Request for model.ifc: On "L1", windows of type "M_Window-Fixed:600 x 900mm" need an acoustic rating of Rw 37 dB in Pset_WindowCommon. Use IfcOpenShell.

First a look at what the model holds.

```python
import ifcopenshell
import ifcopenshell.util.element

model = ifcopenshell.open("model.ifc")
print(model.schema)
storey = next(s for s in model.by_type("IfcBuildingStorey") if s.Name == "L1")
windows = [e for e in ifcopenshell.util.element.get_decomposition(storey) if e.is_a("IfcWindow")]
seen = {}
for e in windows:
    element_type = ifcopenshell.util.element.get_type(e)
    key = (element_type.Name if element_type != e and element_type else None, ifcopenshell.util.element.get_pset(e, "Pset_WindowCommon", "AcousticRating"))
    seen[key] = seen.get(key, 0) + 1
for (name, value), count in sorted(seen.items(), key=str):
    print(count, "x", name, "|", value)
```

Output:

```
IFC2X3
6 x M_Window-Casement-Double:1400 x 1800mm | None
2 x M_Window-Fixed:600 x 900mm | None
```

```python
import ifcopenshell
import ifcopenshell.api.pset
import ifcopenshell.util.element

model = ifcopenshell.open("model.ifc")

storey = next(s for s in model.by_type("IfcBuildingStorey") if s.Name == "L1")
windows = [e for e in ifcopenshell.util.element.get_decomposition(storey) if e.is_a("IfcWindow")]

count = 0
for e in windows:
    element_type = ifcopenshell.util.element.get_type(e)
    if element_type in (None, e) or element_type.Name != "M_Window-Fixed:600 x 900mm":
        continue
    # add_pset returns the element's existing set when there is one.
    pset = ifcopenshell.api.pset.add_pset(model, product=e, name="Pset_WindowCommon")
    ifcopenshell.api.pset.edit_pset(model, pset=pset, properties={"AcousticRating": "Rw 37 dB"})
    count += 1

print(count, "windows updated")

model.write("model_rev.ifc")
```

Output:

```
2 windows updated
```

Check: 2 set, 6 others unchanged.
